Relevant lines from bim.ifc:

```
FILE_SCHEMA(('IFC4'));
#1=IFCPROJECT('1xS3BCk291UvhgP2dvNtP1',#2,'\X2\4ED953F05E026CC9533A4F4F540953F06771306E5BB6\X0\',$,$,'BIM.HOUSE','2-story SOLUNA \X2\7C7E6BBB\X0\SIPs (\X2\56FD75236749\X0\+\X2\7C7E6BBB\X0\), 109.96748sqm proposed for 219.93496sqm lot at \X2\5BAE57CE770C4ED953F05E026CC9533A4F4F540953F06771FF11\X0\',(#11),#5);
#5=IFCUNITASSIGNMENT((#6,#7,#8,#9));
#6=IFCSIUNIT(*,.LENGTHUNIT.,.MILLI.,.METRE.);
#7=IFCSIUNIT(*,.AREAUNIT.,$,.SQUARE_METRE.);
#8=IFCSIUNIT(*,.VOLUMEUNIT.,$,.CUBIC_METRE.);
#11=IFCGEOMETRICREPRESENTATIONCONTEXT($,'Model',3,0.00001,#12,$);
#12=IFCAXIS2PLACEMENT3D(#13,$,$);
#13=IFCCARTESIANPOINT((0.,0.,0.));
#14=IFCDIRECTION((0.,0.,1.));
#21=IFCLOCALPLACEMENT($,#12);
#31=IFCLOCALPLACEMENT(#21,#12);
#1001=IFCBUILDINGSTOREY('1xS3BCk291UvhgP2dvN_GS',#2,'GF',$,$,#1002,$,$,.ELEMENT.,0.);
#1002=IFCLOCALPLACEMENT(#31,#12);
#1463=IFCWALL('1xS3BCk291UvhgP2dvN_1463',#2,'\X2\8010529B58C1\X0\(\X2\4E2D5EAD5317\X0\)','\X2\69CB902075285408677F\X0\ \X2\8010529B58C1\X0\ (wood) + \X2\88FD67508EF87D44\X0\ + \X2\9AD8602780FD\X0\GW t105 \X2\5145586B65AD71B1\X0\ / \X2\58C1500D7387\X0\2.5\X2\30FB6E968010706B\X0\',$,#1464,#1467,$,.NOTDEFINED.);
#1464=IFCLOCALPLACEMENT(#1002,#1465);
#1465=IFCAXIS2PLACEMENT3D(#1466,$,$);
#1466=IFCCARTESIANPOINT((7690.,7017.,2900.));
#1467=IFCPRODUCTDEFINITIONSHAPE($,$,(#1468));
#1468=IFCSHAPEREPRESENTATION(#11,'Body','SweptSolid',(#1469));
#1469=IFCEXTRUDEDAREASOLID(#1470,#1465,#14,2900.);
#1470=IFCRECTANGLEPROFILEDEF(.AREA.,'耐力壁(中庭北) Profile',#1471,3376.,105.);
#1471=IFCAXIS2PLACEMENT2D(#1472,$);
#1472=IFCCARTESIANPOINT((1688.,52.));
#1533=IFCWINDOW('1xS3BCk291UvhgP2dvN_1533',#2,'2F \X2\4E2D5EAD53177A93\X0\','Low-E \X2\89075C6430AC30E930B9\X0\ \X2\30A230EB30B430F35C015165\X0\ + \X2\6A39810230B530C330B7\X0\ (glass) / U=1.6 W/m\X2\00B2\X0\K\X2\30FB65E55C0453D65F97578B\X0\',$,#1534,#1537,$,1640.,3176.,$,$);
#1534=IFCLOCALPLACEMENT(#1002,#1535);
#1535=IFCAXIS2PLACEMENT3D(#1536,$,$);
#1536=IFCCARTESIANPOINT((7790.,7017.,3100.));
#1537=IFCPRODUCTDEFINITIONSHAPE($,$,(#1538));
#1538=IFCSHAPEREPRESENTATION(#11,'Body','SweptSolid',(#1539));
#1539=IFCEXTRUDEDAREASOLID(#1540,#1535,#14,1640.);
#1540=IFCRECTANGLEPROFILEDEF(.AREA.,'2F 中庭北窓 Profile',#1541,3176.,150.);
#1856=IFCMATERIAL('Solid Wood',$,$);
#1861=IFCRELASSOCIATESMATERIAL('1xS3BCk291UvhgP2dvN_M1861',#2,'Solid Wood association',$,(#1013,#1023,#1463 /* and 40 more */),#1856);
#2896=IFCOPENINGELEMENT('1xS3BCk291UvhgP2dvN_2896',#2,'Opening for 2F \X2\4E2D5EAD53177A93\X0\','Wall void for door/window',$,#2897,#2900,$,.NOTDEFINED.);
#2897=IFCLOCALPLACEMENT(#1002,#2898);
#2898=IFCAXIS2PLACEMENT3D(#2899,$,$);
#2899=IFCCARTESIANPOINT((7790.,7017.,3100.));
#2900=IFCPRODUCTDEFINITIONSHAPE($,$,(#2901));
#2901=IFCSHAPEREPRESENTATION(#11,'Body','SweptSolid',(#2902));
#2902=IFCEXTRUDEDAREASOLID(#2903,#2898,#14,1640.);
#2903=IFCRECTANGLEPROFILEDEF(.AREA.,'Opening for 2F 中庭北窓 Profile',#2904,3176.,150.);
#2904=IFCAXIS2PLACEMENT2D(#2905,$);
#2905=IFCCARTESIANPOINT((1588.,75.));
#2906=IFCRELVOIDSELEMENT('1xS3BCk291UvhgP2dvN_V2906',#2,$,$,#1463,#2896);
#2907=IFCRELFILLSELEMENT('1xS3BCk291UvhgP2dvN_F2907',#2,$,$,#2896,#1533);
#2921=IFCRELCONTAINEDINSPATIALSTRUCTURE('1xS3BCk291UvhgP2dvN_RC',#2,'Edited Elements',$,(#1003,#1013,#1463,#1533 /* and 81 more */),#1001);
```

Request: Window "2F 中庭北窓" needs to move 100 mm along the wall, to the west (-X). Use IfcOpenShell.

```python
import ifcopenshell
import ifcopenshell.api.geometry
import ifcopenshell.util.placement
import ifcopenshell.util.unit

model = ifcopenshell.open("bim.ifc")
unit_scale = ifcopenshell.util.unit.calculate_unit_scale(model)

window = model.by_id(1533)
opening = window.FillsVoids[0].RelatingOpeningElement
wall = opening.VoidsElements[0].RelatingBuildingElement

wall_matrix = ifcopenshell.util.placement.get_local_placement(wall.ObjectPlacement)
shift = wall_matrix[:3, 0] * -0.1 / unit_scale
before = ifcopenshell.util.placement.get_local_placement(window.ObjectPlacement)[:3, 3].copy()

# The window is not placed relative to its opening, so move both.
for product in (opening, window):
    matrix = ifcopenshell.util.placement.get_local_placement(product.ObjectPlacement)
    matrix[:3, 3] += shift
    ifcopenshell.api.geometry.edit_object_placement(model, product=product, matrix=matrix, is_si=False)

after = ifcopenshell.util.placement.get_local_placement(window.ObjectPlacement)[:3, 3]
print("window moved by", (after - before).round(3) + 0.0)

model.write("bim_rev.ifc")
```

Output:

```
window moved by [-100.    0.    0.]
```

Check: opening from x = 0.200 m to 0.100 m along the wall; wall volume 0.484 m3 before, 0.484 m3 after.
